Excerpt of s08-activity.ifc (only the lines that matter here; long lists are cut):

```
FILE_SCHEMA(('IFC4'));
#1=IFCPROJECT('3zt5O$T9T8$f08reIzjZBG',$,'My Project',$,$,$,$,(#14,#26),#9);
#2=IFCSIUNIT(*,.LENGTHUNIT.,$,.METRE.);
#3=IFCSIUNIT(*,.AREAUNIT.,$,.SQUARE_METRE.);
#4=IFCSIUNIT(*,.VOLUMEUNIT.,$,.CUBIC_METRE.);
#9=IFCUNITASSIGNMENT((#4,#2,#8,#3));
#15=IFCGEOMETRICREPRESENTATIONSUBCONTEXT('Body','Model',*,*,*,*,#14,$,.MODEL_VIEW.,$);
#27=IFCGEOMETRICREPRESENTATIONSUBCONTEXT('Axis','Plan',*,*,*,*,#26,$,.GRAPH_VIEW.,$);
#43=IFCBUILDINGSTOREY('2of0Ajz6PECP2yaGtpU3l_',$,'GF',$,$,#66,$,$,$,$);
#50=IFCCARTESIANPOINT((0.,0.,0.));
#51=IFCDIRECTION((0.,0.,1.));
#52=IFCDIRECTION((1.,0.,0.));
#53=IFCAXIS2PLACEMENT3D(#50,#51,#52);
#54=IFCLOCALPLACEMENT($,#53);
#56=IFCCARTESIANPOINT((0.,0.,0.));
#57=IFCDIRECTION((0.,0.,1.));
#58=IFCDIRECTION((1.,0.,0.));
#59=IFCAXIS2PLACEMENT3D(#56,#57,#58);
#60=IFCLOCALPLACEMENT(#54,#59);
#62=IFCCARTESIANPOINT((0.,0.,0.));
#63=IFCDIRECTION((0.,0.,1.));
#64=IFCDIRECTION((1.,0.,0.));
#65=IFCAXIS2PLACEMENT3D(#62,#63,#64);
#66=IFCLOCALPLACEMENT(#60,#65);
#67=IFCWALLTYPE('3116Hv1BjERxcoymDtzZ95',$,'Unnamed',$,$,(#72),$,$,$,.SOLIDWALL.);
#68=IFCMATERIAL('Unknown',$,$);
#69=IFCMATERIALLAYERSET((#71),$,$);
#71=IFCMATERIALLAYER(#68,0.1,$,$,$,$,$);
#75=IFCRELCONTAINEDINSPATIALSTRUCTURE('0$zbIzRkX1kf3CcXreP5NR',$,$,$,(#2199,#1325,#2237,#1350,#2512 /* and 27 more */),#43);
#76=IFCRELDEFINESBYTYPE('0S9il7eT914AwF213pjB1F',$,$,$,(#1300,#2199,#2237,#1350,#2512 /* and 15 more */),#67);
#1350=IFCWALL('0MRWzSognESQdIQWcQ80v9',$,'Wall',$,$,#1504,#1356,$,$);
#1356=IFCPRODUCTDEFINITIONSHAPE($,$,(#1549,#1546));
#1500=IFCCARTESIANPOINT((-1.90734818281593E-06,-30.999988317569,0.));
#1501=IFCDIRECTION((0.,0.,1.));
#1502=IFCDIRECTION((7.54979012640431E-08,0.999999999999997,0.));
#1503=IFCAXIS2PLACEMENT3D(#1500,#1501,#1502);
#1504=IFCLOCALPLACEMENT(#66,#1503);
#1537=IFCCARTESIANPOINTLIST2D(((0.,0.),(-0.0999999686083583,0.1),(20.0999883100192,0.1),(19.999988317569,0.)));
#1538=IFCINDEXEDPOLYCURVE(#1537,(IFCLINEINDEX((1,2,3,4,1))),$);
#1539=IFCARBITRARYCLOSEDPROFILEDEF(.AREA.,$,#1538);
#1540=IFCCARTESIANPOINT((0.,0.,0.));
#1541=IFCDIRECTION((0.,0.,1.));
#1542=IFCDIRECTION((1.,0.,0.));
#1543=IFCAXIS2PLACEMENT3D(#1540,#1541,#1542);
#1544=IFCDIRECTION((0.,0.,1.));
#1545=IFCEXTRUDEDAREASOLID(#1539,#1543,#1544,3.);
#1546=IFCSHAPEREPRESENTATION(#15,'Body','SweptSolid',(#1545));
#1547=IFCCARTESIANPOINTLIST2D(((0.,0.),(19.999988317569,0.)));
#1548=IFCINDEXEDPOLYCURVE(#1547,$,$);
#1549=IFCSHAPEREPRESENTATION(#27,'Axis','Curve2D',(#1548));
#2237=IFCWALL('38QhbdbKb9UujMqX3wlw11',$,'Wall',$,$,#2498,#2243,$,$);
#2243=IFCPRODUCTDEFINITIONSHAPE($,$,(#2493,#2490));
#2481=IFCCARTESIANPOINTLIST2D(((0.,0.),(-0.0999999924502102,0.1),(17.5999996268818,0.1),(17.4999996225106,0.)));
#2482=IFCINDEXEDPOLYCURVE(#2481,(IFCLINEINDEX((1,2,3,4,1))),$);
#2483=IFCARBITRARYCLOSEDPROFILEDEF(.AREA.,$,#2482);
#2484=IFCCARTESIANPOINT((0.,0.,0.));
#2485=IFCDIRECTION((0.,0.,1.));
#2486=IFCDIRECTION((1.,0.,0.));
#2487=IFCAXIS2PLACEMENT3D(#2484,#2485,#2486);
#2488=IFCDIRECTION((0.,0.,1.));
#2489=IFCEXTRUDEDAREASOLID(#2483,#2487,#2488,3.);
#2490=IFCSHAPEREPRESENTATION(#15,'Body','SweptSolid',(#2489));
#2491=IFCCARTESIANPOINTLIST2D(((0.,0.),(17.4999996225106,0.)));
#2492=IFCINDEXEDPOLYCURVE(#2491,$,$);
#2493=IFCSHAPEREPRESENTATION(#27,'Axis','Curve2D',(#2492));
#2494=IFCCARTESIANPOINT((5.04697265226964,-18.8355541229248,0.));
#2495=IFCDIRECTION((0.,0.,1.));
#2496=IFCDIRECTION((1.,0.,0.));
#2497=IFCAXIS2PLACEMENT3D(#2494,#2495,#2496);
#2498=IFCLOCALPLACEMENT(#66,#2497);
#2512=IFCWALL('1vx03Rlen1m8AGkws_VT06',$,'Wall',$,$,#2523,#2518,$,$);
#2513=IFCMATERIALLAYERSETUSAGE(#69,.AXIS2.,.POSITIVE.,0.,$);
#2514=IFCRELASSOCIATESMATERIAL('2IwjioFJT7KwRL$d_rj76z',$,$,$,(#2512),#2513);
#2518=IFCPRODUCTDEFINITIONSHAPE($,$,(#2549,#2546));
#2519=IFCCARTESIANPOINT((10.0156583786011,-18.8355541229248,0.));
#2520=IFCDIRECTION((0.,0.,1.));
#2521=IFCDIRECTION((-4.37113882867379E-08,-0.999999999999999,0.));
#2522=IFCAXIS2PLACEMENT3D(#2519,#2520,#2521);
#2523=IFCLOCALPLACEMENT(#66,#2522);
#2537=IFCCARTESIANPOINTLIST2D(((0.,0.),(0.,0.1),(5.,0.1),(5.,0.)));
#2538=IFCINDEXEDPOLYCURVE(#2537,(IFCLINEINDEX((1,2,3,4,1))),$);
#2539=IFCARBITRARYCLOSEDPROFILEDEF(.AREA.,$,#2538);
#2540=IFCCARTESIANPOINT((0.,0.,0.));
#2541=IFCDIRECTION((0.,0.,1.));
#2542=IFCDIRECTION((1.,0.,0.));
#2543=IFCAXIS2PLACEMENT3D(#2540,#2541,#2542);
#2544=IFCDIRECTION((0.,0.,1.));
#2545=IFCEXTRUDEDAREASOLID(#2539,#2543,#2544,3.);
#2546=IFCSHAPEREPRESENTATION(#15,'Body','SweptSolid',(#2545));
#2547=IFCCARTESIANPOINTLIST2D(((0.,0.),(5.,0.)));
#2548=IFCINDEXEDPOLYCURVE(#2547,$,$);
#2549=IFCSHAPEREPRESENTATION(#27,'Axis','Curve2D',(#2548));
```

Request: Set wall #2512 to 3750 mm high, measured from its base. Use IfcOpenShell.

```python
import ifcopenshell
import ifcopenshell.geom
import ifcopenshell.util.representation
import ifcopenshell.util.shape

model = ifcopenshell.open("s08-activity.ifc")
settings = ifcopenshell.geom.settings()


def volume(element):
    """Net volume in cubic metres, openings subtracted."""
    shape = ifcopenshell.geom.create_shape(settings, element)
    return ifcopenshell.util.shape.get_volume(shape.geometry)


wall = model.by_guid("1vx03Rlen1m8AGkws_VT06")
before = volume(wall)

body = ifcopenshell.util.representation.get_representation(wall, "Model", "Body")
solid = body.Items[0]
old_height = solid.Depth
solid.Depth = 3.75
after = volume(wall)

print(f"height {old_height:g} -> {solid.Depth:g}, volume {before:.3f} -> {after:.3f} m3")

model.write("s08-activity_v2.ifc")
```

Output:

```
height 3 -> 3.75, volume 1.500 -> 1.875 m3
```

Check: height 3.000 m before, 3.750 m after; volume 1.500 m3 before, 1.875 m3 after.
